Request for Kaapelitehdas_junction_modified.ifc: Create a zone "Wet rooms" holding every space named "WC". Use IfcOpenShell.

First a look at what the model holds.

```python
import ifcopenshell

model = ifcopenshell.open("Kaapelitehdas_junction_modified.ifc")
print(model.schema)
seen = {}
for space in model.by_type("IfcSpace"):
    seen[space.LongName] = seen.get(space.LongName, 0) + 1
for name, count in sorted(seen.items(), key=str):
    print(count, "x", name)
print("zones:", [z.Name for z in model.by_type("IfcZone")][:20])
```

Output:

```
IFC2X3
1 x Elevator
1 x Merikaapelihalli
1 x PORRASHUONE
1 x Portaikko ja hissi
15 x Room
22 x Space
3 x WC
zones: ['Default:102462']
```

```python
import ifcopenshell
import ifcopenshell.api.group
import ifcopenshell.api.root

model = ifcopenshell.open("Kaapelitehdas_junction_modified.ifc")

names = {"WC"}
spaces = [s for s in model.by_type("IfcSpace") if s.LongName in names]

zone = ifcopenshell.api.root.create_entity(model, ifc_class="IfcZone", name="Wet rooms")
ifcopenshell.api.group.assign_group(model, products=spaces, group=zone)
print(len(spaces), "spaces in", zone.Name)

model.write("Kaapelitehdas_junction_modified_updated.ifc")
```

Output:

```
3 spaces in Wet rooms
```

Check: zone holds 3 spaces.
